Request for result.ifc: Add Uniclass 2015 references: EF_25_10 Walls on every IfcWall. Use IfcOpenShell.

First a look at what the model holds.

```python
import ifcopenshell

model = ifcopenshell.open("result.ifc")
print(model.schema)
print("classifications:", [c.Name for c in model.by_type("IfcClassification")])
for ifc_class in ("IfcDoor", "IfcRoof", "IfcStair", "IfcWall", "IfcWindow"):
    print(ifc_class, len(model.by_type(ifc_class)))
```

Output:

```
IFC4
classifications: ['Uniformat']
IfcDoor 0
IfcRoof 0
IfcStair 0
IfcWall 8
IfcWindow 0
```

```python
import ifcopenshell
import ifcopenshell.api.classification

model = ifcopenshell.open("result.ifc")

system = ifcopenshell.api.classification.add_classification(model, classification="Uniclass 2015")

codes = {
    "IfcWall": ("EF_25_10", "Walls"),
}
for ifc_class, (code, name) in codes.items():
    products = model.by_type(ifc_class)
    ifcopenshell.api.classification.add_reference(
        model, products=products, classification=system, identification=code, name=name
    )
    print(code, len(products))

model.write("result_v2.ifc")
```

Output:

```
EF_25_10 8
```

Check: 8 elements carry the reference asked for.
